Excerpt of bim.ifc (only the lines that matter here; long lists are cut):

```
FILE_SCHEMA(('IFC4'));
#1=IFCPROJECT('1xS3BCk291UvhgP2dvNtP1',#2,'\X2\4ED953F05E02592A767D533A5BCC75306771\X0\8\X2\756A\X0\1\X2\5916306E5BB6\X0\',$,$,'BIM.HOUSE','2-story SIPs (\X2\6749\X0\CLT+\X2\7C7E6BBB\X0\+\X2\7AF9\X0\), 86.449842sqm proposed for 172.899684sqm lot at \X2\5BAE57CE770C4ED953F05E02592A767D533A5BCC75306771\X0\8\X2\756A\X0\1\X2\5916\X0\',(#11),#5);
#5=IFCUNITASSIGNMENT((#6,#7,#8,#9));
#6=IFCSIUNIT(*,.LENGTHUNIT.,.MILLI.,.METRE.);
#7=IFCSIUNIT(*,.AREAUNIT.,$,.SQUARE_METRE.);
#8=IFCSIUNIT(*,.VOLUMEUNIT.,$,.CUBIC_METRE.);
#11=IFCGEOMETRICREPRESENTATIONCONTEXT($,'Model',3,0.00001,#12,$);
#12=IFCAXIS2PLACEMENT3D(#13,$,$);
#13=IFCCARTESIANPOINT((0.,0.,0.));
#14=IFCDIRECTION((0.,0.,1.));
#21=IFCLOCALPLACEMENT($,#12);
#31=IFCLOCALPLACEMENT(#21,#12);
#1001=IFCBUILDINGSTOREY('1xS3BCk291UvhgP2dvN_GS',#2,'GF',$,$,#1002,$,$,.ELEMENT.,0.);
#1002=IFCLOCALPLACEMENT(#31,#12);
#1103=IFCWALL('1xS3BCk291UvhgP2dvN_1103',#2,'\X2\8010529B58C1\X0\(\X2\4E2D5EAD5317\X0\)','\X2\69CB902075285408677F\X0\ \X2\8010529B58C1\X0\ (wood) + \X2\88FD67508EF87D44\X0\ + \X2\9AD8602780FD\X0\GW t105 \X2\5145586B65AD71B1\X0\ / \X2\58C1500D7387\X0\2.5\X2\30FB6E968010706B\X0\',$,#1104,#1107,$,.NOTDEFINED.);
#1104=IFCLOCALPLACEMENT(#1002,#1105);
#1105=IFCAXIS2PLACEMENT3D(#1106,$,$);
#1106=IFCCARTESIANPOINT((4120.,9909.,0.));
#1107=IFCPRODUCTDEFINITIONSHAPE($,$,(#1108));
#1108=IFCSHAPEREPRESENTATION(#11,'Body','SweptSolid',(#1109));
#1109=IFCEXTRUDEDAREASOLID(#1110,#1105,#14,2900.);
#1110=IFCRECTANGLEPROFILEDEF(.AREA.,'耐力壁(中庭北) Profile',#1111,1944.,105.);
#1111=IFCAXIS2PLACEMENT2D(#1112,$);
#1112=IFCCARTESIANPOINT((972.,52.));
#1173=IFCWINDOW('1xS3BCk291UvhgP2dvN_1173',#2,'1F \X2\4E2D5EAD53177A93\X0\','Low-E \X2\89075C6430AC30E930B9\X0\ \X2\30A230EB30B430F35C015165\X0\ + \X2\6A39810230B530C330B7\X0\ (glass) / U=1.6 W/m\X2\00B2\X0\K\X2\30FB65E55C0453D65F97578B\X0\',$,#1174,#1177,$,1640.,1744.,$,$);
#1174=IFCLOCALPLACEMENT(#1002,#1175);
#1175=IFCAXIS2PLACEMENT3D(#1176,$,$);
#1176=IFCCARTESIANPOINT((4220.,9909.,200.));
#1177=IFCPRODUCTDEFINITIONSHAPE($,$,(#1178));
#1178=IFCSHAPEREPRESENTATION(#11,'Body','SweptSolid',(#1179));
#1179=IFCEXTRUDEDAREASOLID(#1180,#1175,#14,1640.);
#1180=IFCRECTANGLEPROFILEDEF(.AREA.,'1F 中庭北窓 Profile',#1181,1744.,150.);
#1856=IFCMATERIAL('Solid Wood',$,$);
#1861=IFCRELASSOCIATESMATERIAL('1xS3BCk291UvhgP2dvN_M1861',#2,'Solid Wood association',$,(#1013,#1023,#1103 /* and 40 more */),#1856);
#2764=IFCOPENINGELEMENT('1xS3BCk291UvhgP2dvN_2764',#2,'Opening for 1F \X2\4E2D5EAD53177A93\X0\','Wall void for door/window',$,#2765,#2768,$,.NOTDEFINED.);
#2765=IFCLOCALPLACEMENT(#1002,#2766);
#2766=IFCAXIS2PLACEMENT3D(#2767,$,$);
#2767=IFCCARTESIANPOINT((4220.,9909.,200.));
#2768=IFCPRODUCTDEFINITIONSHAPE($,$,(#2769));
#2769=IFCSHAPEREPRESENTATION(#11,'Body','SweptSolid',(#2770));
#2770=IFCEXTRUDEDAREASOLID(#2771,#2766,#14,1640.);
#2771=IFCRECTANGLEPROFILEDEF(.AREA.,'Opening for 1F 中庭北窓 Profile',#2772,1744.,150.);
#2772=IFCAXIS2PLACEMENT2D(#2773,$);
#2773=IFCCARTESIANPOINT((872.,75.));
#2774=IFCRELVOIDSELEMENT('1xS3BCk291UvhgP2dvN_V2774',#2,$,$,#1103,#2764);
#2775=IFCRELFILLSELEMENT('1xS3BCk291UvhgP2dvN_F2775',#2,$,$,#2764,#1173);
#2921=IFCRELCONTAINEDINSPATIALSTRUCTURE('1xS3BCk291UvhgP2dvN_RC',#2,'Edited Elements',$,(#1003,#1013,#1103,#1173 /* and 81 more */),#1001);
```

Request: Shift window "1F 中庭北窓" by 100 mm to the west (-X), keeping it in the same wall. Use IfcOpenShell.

```python
import ifcopenshell
import ifcopenshell.api.geometry
import ifcopenshell.util.placement
import ifcopenshell.util.unit

model = ifcopenshell.open("bim.ifc")
unit_scale = ifcopenshell.util.unit.calculate_unit_scale(model)

window = model.by_guid("1xS3BCk291UvhgP2dvN_1173")
opening = window.FillsVoids[0].RelatingOpeningElement
wall = opening.VoidsElements[0].RelatingBuildingElement

wall_matrix = ifcopenshell.util.placement.get_local_placement(wall.ObjectPlacement)
shift = wall_matrix[:3, 0] * -0.1 / unit_scale
before = ifcopenshell.util.placement.get_local_placement(window.ObjectPlacement)[:3, 3].copy()

# The window is not placed relative to its opening, so move both.
for product in (opening, window):
    matrix = ifcopenshell.util.placement.get_local_placement(product.ObjectPlacement)
    matrix[:3, 3] += shift
    ifcopenshell.api.geometry.edit_object_placement(model, product=product, matrix=matrix, is_si=False)

after = ifcopenshell.util.placement.get_local_placement(window.ObjectPlacement)[:3, 3]
print("window moved by", (after - before).round(3) + 0.0)

model.write("bim_v2.ifc")
```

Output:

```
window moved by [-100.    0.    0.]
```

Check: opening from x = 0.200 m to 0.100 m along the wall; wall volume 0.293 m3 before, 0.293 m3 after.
